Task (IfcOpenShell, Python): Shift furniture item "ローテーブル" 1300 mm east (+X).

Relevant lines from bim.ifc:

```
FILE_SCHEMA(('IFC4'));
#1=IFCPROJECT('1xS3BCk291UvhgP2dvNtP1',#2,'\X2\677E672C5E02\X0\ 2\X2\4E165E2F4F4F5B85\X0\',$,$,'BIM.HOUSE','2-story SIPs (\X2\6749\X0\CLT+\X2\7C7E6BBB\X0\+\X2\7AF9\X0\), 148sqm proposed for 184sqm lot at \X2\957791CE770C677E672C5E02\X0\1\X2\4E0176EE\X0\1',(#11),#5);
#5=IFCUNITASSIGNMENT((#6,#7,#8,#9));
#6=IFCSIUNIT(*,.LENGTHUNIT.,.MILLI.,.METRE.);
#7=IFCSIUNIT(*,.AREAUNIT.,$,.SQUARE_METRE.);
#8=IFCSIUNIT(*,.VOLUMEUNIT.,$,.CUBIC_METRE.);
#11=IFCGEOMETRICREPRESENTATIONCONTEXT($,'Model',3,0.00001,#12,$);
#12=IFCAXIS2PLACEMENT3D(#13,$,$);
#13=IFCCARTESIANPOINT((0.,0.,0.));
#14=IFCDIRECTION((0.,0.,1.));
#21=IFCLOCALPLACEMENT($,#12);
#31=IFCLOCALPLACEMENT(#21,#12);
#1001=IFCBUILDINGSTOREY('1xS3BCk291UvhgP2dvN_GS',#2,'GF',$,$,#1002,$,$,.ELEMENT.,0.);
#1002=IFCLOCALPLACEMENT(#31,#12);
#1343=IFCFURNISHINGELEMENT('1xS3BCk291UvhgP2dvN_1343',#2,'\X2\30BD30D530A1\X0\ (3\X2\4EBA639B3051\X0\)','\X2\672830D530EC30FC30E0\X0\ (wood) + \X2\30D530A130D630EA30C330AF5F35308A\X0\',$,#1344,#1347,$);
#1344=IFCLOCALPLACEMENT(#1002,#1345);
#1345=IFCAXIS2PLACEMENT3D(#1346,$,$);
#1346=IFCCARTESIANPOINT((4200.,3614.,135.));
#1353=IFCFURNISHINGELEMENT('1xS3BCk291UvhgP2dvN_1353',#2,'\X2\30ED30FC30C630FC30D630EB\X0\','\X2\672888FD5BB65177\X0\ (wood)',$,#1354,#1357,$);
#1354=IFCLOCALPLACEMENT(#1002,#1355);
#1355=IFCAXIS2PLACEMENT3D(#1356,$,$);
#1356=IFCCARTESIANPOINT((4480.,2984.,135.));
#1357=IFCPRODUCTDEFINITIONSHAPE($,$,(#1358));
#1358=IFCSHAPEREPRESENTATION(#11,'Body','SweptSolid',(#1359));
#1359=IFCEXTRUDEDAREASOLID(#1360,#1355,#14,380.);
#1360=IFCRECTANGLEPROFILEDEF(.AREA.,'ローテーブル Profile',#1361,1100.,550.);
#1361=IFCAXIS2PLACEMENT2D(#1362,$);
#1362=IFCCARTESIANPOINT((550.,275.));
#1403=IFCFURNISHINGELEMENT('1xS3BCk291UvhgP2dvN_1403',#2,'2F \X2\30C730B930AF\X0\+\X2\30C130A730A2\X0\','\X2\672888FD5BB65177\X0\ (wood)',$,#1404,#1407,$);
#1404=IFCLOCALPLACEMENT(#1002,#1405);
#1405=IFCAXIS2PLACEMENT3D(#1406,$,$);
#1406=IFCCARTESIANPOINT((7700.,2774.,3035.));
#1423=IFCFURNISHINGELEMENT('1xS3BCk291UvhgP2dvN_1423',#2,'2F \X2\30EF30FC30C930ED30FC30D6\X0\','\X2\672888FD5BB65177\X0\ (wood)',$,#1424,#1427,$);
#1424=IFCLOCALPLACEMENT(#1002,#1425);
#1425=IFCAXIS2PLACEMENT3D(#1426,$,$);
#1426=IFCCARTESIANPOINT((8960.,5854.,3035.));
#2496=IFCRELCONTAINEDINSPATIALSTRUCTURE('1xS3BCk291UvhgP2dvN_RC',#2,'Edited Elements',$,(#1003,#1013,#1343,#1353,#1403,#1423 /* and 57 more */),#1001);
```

```python
import ifcopenshell
import ifcopenshell.api.geometry
import ifcopenshell.util.placement

model = ifcopenshell.open("bim.ifc")

item = model.by_guid("1xS3BCk291UvhgP2dvN_1353")
matrix = ifcopenshell.util.placement.get_local_placement(item.ObjectPlacement)
matrix[0, 3] += 1300.0
ifcopenshell.api.geometry.edit_object_placement(model, product=item, matrix=matrix, is_si=False)

print(ifcopenshell.util.placement.get_local_placement(item.ObjectPlacement).round(3) + 0.0)

model.write("bim_updated.ifc")
```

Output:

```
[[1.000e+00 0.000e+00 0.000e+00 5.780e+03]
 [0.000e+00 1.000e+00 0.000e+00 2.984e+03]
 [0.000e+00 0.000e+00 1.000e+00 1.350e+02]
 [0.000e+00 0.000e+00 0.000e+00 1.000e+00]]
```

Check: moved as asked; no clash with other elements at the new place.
